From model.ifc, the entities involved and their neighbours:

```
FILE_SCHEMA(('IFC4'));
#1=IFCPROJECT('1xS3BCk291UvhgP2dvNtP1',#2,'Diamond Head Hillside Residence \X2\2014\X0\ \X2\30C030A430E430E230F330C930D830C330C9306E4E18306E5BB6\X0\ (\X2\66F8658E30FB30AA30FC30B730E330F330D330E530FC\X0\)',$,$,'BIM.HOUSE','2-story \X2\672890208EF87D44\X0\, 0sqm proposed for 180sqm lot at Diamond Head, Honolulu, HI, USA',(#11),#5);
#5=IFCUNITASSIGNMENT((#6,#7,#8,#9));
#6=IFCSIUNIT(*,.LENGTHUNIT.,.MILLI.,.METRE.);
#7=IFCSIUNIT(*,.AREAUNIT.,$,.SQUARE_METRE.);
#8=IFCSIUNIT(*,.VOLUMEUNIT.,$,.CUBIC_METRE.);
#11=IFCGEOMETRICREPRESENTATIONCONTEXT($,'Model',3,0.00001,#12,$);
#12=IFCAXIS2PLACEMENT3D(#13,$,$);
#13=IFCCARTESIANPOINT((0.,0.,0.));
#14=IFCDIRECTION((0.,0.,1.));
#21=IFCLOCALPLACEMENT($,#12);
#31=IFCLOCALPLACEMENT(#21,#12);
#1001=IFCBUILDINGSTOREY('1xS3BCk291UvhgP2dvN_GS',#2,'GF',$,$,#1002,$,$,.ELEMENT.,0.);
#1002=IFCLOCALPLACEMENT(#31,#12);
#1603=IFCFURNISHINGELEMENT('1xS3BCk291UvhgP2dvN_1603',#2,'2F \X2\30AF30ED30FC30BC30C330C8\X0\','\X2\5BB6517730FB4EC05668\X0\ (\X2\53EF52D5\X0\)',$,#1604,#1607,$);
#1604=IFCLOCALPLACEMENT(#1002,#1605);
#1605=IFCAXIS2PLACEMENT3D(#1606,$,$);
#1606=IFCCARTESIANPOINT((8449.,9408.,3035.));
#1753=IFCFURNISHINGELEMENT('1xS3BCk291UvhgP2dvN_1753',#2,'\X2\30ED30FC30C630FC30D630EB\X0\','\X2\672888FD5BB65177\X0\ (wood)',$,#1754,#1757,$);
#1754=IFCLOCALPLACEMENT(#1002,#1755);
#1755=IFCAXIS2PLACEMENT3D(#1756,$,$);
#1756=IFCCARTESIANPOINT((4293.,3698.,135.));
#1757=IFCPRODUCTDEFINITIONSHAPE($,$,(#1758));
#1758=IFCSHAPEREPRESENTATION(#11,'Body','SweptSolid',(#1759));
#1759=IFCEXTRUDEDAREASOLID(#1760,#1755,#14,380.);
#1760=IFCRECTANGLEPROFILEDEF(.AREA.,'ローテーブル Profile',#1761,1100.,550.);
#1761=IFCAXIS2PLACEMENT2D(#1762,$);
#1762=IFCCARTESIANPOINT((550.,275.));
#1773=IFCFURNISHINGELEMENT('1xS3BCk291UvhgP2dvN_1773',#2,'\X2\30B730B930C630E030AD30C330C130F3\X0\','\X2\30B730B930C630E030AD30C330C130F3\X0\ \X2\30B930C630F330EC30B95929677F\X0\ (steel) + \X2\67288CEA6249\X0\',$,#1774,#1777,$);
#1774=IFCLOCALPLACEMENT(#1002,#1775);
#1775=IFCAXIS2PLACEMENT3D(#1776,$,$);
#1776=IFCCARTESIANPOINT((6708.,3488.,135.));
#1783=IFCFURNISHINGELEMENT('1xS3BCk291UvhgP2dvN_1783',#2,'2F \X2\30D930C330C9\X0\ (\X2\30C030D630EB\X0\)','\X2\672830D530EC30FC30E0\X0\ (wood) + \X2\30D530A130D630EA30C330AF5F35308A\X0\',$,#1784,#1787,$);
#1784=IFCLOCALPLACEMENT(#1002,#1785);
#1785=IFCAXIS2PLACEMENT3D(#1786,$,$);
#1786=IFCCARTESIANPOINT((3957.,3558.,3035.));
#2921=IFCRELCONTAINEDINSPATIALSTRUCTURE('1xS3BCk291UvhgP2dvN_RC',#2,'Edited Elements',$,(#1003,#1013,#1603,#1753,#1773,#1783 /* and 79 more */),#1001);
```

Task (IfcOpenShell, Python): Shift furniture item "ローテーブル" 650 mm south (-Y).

```python
import ifcopenshell
import ifcopenshell.api.geometry
import ifcopenshell.util.placement

model = ifcopenshell.open("model.ifc")

item = model.by_id(1753)
matrix = ifcopenshell.util.placement.get_local_placement(item.ObjectPlacement)
matrix[1, 3] -= 650.0
ifcopenshell.api.geometry.edit_object_placement(model, product=item, matrix=matrix, is_si=False)

print(ifcopenshell.util.placement.get_local_placement(item.ObjectPlacement).round(3) + 0.0)

model.write("model-out.ifc")
```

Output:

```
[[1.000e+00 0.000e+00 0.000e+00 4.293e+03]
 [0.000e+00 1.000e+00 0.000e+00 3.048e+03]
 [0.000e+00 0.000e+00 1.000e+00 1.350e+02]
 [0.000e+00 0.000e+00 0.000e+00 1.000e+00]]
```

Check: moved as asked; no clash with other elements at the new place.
